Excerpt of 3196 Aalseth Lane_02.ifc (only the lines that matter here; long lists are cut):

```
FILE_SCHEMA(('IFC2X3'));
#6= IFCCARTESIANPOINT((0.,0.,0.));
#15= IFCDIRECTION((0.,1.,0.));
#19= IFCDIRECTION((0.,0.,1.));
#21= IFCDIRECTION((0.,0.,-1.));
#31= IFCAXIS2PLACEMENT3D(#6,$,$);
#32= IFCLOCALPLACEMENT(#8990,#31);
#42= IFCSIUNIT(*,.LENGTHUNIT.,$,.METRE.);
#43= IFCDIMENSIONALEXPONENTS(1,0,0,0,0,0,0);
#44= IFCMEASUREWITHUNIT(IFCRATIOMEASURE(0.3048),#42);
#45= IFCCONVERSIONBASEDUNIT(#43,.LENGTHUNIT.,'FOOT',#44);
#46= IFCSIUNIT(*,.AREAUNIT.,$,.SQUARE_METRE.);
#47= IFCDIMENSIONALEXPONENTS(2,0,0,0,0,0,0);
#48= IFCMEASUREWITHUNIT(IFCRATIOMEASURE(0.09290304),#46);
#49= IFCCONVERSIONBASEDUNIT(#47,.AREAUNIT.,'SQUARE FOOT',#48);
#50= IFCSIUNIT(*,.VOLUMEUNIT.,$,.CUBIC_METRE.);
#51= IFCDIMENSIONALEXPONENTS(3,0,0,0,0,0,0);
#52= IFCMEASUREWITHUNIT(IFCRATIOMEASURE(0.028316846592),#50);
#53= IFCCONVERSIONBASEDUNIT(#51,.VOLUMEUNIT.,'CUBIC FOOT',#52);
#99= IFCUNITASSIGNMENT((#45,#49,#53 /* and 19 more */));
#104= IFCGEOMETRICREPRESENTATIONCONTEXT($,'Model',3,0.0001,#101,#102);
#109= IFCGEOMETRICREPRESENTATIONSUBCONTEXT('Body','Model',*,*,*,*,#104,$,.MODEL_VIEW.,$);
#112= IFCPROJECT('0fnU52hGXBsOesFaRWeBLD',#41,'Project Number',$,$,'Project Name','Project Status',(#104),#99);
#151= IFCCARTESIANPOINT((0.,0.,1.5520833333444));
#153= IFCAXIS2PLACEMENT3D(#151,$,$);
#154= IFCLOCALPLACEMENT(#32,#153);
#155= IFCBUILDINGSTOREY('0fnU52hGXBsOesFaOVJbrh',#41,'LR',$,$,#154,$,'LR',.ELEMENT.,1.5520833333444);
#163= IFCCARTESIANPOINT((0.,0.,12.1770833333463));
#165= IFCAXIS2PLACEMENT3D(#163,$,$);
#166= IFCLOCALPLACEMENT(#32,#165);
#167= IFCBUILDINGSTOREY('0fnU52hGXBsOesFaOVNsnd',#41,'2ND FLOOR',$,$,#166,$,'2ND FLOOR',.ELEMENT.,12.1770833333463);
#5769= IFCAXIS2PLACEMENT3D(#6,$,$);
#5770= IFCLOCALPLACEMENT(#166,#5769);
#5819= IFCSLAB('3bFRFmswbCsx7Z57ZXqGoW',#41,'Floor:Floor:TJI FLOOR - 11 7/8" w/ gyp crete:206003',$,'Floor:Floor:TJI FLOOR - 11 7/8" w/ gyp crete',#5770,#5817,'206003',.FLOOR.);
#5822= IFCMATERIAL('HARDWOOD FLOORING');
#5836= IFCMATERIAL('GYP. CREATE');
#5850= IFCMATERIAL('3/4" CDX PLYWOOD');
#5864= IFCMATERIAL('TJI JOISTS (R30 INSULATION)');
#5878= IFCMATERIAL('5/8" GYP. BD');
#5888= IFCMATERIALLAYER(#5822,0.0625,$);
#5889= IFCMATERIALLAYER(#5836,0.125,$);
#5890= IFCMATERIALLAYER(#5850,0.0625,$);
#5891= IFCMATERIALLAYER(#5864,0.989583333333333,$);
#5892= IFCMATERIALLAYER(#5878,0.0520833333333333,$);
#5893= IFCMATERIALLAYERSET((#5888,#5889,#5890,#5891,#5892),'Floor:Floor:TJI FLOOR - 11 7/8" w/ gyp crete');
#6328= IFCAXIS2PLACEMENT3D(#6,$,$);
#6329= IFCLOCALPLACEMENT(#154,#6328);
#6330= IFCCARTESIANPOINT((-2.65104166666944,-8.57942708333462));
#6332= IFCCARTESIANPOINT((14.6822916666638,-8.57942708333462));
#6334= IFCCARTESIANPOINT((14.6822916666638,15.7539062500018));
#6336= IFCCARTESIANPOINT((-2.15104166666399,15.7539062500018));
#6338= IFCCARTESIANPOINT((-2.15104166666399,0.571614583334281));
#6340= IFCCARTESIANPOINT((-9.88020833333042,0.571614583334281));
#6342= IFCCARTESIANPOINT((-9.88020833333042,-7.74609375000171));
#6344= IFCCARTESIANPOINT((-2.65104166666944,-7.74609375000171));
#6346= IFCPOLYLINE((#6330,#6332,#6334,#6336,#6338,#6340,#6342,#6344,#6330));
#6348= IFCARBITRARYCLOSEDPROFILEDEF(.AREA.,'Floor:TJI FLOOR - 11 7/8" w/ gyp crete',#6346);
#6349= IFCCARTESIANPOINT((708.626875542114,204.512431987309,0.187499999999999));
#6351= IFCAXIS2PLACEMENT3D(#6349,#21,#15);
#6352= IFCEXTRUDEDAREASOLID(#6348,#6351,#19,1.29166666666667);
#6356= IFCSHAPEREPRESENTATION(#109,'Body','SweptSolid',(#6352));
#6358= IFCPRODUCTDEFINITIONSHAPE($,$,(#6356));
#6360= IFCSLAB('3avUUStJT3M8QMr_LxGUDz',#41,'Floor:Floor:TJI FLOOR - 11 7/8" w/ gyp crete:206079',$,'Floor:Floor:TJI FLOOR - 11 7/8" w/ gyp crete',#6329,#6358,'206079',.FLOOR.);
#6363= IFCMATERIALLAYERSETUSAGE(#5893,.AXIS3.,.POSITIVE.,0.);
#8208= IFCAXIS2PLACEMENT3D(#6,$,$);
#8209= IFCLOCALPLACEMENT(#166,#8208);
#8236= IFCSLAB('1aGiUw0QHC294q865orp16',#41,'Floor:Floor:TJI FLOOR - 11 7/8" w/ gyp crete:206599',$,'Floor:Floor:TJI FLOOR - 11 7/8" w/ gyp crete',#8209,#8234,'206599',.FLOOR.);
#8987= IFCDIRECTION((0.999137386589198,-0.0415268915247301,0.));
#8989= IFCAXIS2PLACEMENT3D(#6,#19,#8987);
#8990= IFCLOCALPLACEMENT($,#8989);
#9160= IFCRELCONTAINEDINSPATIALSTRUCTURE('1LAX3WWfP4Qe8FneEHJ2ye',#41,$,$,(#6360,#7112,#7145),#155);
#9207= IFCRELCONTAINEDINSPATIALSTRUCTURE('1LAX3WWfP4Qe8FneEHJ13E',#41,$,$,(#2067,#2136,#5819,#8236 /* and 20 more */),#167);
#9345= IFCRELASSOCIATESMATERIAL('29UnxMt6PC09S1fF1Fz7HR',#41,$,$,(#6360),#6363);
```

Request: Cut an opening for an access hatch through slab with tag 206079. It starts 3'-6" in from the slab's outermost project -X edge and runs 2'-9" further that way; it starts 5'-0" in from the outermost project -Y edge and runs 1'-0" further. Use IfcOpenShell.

```python
import numpy as np
import ifcopenshell
import ifcopenshell.api.feature
import ifcopenshell.api.geometry
import ifcopenshell.api.root
import ifcopenshell.geom
import ifcopenshell.util.placement
import ifcopenshell.util.representation
import ifcopenshell.util.shape
import ifcopenshell.util.unit

model = ifcopenshell.open("3196 Aalseth Lane_02.ifc")
unit_scale = ifcopenshell.util.unit.calculate_unit_scale(model)
settings = ifcopenshell.geom.settings()


def volume(element):
    """Net volume in cubic metres, openings subtracted."""
    shape = ifcopenshell.geom.create_shape(settings, element)
    return ifcopenshell.util.shape.get_volume(shape.geometry)


slab = model.by_id(6360)
before = volume(slab)

# Extent in the slab's own axes, in metres. The edges named are its -X and -Y sides.
slab_shape = ifcopenshell.geom.create_shape(settings, slab)
vertices = ifcopenshell.util.shape.get_vertices(slab_shape.geometry)
x_min, y_min, bottom = vertices.min(axis=0)
top = vertices[:, 2].max()

opening = ifcopenshell.api.root.create_entity(model, ifc_class="IfcOpeningElement", name="Access hatch opening")
context = ifcopenshell.util.representation.get_context(model, "Model", "Body", "MODEL_VIEW")
width, depth = 0.8382, 0.3048
outline = [(0.0, 0.0), (width, 0.0), (width, depth), (0.0, depth), (0.0, 0.0)]
# Overshoot both faces by 50 mm so the cut is clean.
shape = ifcopenshell.api.geometry.add_slab_representation(
    model, context=context, depth=top - bottom + 0.1, polyline=outline
)
ifcopenshell.api.geometry.assign_representation(model, product=opening, representation=shape)

matrix = ifcopenshell.util.placement.get_local_placement(slab.ObjectPlacement)
matrix[:, 3] = matrix @ np.append(np.array([x_min + 1.0668, y_min + 1.524, bottom - 0.05]) / unit_scale, 1.0)
ifcopenshell.api.geometry.edit_object_placement(model, product=opening, matrix=matrix, is_si=False)
ifcopenshell.api.feature.add_feature(model, feature=opening, element=slab)

after = volume(slab)

print(f"slab volume {before:.3f} -> {after:.3f} m3")

model.write("3196 Aalseth Lane_02_v2.ifc")
```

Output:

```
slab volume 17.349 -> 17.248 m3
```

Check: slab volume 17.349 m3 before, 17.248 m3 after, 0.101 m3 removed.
